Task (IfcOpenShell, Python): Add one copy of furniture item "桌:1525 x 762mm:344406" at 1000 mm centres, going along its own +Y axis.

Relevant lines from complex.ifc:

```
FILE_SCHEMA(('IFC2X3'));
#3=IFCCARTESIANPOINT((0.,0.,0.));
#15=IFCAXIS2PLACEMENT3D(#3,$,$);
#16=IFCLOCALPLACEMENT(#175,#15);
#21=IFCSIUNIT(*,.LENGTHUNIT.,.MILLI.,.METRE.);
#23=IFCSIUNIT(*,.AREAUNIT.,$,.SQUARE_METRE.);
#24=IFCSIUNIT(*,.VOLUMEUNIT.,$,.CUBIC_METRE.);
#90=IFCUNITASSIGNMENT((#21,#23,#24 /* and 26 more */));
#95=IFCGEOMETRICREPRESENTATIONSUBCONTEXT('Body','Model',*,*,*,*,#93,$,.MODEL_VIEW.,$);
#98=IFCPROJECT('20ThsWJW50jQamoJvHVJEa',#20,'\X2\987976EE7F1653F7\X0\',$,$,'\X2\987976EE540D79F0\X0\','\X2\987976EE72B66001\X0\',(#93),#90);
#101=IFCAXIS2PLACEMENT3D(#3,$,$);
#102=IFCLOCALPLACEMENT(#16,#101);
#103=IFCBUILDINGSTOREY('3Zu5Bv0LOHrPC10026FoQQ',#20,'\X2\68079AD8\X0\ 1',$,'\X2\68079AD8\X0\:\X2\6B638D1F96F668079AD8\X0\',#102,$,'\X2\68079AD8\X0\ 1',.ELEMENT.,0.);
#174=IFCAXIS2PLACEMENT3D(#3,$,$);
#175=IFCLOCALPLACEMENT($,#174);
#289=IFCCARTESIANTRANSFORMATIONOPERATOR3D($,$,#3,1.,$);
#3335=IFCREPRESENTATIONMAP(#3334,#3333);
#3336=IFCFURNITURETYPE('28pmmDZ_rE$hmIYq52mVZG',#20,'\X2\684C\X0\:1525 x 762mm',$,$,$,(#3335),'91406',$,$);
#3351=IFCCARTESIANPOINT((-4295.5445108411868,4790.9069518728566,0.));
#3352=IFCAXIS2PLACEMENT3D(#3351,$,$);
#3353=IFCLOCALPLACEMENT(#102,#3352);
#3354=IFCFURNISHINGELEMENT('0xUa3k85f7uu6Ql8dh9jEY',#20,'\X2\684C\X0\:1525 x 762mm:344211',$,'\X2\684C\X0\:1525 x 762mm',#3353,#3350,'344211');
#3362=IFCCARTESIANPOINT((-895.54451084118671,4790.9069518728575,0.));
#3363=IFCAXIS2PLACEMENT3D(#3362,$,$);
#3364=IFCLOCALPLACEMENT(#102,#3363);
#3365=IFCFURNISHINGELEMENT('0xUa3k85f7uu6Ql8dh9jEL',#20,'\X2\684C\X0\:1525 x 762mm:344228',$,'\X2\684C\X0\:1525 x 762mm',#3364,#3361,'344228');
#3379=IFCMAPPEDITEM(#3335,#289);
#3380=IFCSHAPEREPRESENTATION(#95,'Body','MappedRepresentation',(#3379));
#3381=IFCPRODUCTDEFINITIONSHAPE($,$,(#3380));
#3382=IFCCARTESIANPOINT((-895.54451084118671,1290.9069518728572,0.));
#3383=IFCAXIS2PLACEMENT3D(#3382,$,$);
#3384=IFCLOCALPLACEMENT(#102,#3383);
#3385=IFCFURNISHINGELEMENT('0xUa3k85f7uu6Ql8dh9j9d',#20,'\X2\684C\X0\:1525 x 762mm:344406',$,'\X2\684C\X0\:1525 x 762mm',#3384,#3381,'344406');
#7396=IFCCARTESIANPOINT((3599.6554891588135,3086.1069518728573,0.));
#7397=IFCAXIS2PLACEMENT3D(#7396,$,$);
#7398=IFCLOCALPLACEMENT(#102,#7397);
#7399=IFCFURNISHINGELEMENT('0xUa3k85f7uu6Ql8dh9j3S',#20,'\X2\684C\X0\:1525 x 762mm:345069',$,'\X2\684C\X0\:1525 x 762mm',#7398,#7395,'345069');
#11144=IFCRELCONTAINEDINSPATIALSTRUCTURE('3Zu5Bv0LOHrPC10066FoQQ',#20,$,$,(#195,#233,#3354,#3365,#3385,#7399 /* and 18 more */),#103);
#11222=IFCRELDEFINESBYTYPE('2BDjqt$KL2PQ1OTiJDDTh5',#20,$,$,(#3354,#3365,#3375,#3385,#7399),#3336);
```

```python
import ifcopenshell
import ifcopenshell.api.geometry
import ifcopenshell.api.root
import ifcopenshell.util.element
import ifcopenshell.util.placement
import ifcopenshell.util.unit

model = ifcopenshell.open("complex.ifc")
unit_scale = ifcopenshell.util.unit.calculate_unit_scale(model)


def reuse_history(source, copy):
    """copy_class also copies each property set's owner history, people and application; keep the originals."""
    for rel in copy.IsDefinedBy:
        if rel.is_a("IfcRelDefinesByProperties") and (history := rel.RelatingPropertyDefinition.OwnerHistory):
            rel.RelatingPropertyDefinition.OwnerHistory = source.OwnerHistory
            ifcopenshell.util.element.remove_deep2(model, history)


source = model.by_guid("0xUa3k85f7uu6Ql8dh9j9d")
base = ifcopenshell.util.placement.get_local_placement(source.ObjectPlacement)
step = base[:3, 1] * 1 / unit_scale

for i in range(1, 2):
    copy = ifcopenshell.api.root.copy_class(model, product=source)
    copy.Representation = ifcopenshell.util.element.copy_deep(
        model, source.Representation, exclude=["IfcGeometricRepresentationContext", "IfcRepresentationMap"]
    )
    copy.Name = "桌:1525 x 762mm"
    copy.Tag = None
    reuse_history(source, copy)
    matrix = base.copy()
    matrix[:3, 3] += i * step
    print("added at", matrix[:3, 3].round(3) + 0.0)
    ifcopenshell.api.geometry.edit_object_placement(model, product=copy, matrix=matrix, is_si=False)

model.write("complex_rev.ifc")
```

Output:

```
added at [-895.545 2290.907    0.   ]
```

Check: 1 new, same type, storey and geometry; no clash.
